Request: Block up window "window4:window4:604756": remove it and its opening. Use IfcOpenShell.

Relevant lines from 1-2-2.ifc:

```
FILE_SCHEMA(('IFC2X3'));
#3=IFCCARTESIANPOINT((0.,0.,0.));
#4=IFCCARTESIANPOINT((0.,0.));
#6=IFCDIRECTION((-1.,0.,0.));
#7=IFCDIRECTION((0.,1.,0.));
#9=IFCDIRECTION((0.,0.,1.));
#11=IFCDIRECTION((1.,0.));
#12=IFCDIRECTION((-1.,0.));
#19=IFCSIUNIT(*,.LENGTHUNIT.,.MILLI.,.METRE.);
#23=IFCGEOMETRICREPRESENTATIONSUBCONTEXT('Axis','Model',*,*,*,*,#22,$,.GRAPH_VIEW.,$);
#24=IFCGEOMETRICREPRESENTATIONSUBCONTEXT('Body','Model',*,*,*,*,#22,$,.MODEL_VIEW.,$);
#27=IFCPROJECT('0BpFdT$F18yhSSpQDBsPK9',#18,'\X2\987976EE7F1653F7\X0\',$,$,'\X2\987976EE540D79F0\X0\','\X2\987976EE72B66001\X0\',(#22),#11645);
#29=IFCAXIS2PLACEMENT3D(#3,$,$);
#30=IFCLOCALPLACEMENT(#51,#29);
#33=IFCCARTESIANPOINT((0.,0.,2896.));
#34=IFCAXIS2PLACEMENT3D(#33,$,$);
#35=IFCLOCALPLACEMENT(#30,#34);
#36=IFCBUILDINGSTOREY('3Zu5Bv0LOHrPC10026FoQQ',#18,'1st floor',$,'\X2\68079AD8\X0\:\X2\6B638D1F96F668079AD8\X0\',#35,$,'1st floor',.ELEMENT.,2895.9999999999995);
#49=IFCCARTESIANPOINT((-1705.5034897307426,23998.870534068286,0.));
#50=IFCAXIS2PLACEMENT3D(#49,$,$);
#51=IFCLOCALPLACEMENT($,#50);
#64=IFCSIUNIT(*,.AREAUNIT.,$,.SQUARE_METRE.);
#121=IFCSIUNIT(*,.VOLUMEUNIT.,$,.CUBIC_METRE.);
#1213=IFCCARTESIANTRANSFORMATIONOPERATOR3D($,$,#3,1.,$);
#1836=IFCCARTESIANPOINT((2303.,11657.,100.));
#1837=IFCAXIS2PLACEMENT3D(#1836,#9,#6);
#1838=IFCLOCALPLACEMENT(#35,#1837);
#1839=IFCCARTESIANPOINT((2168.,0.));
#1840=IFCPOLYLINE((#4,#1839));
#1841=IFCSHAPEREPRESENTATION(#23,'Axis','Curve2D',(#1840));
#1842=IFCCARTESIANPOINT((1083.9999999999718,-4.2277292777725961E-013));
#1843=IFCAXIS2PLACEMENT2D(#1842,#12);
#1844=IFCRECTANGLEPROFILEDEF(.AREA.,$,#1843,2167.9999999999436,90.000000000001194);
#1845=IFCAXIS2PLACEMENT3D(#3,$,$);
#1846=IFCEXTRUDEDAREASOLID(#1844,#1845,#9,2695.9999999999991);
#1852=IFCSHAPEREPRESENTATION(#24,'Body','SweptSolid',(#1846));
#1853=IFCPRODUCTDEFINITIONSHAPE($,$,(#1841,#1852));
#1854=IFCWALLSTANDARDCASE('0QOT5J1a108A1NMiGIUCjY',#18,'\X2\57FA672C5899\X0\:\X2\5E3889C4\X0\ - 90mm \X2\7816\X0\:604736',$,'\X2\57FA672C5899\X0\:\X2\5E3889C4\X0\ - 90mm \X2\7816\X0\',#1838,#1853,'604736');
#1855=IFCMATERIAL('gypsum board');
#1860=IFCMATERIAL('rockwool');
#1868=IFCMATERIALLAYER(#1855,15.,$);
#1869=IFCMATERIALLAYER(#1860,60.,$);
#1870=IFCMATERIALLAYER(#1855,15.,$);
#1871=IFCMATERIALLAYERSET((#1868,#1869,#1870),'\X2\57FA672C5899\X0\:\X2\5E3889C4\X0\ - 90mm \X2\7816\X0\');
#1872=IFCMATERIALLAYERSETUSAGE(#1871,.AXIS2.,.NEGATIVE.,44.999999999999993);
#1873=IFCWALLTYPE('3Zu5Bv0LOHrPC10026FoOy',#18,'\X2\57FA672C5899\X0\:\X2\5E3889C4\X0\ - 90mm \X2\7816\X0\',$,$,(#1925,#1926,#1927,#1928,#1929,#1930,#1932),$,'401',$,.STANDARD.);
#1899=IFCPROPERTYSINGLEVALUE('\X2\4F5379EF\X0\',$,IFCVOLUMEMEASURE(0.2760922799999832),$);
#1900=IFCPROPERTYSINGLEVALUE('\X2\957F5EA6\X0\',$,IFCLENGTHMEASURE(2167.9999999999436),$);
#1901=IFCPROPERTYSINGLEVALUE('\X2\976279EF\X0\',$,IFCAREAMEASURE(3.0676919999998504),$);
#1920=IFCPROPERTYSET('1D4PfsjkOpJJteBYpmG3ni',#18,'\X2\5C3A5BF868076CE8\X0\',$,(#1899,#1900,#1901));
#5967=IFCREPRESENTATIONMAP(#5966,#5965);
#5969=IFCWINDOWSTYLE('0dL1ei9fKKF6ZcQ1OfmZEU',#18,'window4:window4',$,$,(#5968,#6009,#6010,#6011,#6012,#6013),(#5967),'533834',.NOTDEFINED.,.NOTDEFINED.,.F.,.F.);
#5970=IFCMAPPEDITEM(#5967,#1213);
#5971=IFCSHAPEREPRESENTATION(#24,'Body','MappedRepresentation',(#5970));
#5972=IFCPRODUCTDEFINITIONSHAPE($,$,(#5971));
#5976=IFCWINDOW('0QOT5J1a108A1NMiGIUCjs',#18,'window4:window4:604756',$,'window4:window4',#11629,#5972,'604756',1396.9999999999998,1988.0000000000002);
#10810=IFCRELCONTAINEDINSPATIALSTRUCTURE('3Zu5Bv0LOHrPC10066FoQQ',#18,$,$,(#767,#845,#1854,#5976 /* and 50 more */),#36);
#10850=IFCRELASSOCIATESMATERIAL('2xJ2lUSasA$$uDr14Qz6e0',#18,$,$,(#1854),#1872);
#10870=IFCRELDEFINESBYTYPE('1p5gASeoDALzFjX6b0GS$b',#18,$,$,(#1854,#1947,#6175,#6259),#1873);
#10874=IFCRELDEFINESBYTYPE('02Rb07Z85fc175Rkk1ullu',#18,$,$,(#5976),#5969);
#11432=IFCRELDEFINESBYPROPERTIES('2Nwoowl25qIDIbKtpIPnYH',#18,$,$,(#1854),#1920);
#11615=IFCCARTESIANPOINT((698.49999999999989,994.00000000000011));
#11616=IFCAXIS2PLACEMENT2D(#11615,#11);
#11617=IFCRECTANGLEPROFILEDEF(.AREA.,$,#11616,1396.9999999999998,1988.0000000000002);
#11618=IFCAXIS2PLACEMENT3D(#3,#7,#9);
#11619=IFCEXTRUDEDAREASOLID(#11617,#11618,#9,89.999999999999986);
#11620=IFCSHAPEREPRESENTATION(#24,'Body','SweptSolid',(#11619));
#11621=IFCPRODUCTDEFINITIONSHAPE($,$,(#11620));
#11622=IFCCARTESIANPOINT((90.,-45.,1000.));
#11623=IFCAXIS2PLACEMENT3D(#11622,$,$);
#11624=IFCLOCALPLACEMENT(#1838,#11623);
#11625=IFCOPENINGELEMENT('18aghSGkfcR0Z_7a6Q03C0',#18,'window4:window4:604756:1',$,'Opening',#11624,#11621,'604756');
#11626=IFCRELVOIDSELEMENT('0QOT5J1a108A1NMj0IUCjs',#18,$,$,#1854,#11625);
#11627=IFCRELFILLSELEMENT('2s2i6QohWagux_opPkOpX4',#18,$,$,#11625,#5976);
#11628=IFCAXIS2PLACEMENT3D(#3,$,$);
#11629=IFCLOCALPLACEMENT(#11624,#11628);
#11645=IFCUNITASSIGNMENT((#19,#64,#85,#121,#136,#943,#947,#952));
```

```python
import ifcopenshell
import ifcopenshell.api.feature
import ifcopenshell.api.pset
import ifcopenshell.api.root
import ifcopenshell.geom
import ifcopenshell.util.element
import ifcopenshell.util.shape
import ifcopenshell.util.unit

model = ifcopenshell.open("1-2-2.ifc")
area_scale = ifcopenshell.util.unit.calculate_unit_scale(model, "AREAUNIT")
volume_scale = ifcopenshell.util.unit.calculate_unit_scale(model, "VOLUMEUNIT")
settings = ifcopenshell.geom.settings()


def volume(element):
    """Net volume in cubic metres, openings subtracted."""
    shape = ifcopenshell.geom.create_shape(settings, element)
    return ifcopenshell.util.shape.get_volume(shape.geometry)


window = model.by_id(5976)
opening = window.FillsVoids[0].RelatingOpeningElement
wall = opening.VoidsElements[0].RelatingBuildingElement
before = volume(wall)

ifcopenshell.api.root.remove_product(model, product=window)
ifcopenshell.api.feature.remove_feature(model, feature=opening)

after = volume(wall)
thickness = 0.09  # wall thickness in metres

# Update the wall's stored quantities.
pset = model.by_id(ifcopenshell.util.element.get_pset(wall, "尺寸标注", should_inherit=False)["id"])
ifcopenshell.api.pset.edit_pset(model, pset=pset, properties={
    "体积": model.create_entity("IfcVolumeMeasure", after / volume_scale),
    "面积": model.create_entity("IfcAreaMeasure", after / thickness / area_scale),
})

print(f"wall volume {before:.3f} -> {after:.3f} m3")

model.write("1-2-2-out.ifc")
```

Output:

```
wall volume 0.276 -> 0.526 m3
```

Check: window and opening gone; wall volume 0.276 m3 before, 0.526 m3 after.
